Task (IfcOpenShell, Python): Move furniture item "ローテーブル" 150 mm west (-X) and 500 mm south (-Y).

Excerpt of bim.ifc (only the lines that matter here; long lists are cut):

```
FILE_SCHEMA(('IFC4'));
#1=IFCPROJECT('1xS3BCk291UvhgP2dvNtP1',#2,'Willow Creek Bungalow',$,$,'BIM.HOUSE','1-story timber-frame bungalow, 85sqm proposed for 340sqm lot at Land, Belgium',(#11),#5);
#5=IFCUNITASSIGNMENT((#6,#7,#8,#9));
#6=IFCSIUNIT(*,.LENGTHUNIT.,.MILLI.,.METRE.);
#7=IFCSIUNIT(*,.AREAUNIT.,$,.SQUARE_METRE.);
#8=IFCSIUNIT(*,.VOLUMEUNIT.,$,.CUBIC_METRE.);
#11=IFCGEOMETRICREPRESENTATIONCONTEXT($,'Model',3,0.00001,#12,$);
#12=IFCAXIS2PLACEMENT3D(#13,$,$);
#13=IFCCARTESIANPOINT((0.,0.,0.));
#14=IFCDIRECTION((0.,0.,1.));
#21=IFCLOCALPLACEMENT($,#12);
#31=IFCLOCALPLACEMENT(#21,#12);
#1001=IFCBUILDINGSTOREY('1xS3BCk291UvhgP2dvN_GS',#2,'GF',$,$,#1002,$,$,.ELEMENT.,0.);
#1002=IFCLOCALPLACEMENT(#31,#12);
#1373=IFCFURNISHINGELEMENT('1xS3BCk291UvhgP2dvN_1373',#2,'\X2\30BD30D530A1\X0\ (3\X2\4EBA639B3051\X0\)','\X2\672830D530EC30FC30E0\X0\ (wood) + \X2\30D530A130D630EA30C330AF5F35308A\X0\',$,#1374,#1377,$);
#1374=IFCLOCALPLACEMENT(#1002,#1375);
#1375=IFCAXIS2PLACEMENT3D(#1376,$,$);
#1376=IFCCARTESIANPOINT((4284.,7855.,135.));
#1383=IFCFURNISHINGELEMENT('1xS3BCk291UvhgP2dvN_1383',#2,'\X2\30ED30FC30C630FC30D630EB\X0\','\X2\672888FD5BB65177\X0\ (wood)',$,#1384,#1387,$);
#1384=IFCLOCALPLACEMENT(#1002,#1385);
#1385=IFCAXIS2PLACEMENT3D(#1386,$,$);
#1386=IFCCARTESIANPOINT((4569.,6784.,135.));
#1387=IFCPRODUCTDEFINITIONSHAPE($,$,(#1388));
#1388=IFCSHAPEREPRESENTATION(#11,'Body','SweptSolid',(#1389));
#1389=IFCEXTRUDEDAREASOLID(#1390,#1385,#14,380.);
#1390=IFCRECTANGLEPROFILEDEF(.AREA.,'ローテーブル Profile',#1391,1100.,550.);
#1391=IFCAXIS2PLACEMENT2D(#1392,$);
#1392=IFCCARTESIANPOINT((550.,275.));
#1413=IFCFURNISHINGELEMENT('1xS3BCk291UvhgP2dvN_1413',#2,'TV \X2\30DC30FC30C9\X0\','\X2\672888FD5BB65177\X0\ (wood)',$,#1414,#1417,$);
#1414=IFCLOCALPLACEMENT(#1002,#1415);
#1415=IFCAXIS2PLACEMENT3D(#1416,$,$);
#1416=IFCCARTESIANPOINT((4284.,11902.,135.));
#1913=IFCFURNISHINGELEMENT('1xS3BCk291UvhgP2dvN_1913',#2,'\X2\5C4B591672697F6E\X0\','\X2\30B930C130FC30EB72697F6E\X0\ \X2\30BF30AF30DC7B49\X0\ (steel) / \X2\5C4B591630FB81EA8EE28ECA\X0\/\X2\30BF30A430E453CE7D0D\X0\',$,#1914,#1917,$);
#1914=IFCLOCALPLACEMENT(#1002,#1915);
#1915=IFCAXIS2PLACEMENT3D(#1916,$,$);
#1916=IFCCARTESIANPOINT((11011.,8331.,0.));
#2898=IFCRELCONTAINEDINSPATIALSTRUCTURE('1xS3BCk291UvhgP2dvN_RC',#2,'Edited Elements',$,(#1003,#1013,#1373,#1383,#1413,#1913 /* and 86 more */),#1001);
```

```python
import ifcopenshell
import ifcopenshell.api.geometry
import ifcopenshell.util.placement
import ifcopenshell.util.unit

model = ifcopenshell.open("bim.ifc")
unit_scale = ifcopenshell.util.unit.calculate_unit_scale(model)

item = model.by_guid("1xS3BCk291UvhgP2dvN_1383")
matrix = ifcopenshell.util.placement.get_local_placement(item.ObjectPlacement)
matrix[0, 3] -= 0.15 / unit_scale
matrix[1, 3] -= 0.5 / unit_scale
ifcopenshell.api.geometry.edit_object_placement(model, product=item, matrix=matrix, is_si=False)

print(ifcopenshell.util.placement.get_local_placement(item.ObjectPlacement).round(3) + 0.0)

model.write("bim_rev.ifc")
```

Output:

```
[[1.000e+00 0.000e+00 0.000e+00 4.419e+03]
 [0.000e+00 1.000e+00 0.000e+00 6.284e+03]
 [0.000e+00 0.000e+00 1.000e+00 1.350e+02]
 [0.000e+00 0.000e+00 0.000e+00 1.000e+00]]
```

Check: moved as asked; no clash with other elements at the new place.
